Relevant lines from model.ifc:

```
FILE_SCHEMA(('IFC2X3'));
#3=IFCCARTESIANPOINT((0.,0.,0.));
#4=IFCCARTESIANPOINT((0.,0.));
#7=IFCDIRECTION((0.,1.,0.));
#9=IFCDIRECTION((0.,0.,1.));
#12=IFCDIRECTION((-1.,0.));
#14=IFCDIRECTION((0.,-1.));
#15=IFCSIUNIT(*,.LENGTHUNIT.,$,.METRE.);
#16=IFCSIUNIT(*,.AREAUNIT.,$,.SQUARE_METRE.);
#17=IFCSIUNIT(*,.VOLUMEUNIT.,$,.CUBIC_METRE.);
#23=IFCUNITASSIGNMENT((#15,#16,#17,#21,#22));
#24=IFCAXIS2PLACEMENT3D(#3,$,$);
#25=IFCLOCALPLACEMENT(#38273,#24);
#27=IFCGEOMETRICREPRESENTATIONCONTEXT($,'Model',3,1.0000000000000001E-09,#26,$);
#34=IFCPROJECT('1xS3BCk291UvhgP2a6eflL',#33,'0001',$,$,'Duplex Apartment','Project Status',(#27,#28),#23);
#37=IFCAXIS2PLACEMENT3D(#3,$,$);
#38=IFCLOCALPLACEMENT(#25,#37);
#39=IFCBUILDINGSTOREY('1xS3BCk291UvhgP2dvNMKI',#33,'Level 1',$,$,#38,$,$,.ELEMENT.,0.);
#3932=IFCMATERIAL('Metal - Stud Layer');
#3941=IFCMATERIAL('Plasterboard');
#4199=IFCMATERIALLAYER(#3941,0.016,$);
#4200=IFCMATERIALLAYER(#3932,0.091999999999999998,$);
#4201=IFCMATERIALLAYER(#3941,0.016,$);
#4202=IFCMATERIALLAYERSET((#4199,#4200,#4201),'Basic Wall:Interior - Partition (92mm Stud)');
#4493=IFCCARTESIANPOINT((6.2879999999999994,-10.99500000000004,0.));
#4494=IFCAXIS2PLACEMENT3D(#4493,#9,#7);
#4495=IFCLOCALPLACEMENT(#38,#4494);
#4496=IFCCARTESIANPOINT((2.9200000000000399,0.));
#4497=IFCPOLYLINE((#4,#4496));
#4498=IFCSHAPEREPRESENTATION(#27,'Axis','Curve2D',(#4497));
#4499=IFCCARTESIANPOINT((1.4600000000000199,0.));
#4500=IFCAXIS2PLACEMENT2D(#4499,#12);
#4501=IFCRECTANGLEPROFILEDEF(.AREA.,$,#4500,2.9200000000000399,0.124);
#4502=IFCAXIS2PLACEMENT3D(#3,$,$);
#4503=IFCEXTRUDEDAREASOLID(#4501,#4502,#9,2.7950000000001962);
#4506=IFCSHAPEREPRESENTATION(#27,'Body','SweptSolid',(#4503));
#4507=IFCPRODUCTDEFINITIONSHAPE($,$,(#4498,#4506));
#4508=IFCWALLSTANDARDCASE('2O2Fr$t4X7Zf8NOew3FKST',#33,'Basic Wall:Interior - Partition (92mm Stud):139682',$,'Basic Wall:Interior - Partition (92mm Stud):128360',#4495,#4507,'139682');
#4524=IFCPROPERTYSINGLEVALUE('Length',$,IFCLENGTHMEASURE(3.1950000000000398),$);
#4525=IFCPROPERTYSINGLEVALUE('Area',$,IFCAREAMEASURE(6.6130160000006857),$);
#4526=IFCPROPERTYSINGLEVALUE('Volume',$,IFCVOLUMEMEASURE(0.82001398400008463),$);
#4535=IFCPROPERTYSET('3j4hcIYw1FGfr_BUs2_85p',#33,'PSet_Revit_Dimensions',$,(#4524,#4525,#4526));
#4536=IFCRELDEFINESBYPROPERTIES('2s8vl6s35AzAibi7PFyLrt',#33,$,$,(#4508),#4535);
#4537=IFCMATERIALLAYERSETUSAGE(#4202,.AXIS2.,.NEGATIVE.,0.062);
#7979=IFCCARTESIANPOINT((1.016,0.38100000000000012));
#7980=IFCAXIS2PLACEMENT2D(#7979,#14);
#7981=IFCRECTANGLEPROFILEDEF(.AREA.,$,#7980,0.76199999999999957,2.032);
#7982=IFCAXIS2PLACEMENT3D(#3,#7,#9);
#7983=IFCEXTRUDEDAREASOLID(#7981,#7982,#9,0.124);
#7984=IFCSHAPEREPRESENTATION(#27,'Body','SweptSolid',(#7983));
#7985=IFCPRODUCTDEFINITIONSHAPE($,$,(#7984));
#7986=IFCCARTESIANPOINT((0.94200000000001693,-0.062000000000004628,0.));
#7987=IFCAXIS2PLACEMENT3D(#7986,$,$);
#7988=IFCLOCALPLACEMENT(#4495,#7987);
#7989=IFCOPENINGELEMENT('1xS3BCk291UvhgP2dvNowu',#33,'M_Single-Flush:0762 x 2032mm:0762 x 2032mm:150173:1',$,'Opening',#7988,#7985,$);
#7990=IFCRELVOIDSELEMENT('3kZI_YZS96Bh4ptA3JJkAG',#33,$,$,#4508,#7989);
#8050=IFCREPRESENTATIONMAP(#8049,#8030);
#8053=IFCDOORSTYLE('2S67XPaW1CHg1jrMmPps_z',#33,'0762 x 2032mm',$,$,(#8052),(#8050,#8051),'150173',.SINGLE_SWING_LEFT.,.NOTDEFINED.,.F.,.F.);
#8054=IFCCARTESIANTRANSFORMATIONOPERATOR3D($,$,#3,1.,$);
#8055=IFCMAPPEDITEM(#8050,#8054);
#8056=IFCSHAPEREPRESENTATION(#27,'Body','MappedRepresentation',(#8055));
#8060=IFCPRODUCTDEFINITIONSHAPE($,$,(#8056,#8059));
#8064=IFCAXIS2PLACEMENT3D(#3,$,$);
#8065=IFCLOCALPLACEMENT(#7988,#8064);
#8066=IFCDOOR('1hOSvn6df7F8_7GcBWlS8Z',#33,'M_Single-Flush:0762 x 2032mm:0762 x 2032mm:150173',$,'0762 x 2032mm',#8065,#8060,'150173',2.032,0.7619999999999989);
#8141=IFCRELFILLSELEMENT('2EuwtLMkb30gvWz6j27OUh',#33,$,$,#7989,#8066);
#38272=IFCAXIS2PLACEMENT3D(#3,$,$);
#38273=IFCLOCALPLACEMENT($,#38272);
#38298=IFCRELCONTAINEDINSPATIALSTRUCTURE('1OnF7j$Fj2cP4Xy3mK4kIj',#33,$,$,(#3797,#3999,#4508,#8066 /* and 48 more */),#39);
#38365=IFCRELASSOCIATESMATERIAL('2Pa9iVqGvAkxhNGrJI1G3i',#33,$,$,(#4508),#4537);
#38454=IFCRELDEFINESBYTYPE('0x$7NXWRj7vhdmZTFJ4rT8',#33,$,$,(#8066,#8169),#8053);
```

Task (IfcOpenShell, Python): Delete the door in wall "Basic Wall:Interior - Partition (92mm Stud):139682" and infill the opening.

```python
import ifcopenshell
import ifcopenshell.api.feature
import ifcopenshell.api.pset
import ifcopenshell.api.root
import ifcopenshell.geom
import ifcopenshell.util.element
import ifcopenshell.util.shape
import ifcopenshell.util.unit

model = ifcopenshell.open("model.ifc")
area_scale = ifcopenshell.util.unit.calculate_unit_scale(model, "AREAUNIT")
volume_scale = ifcopenshell.util.unit.calculate_unit_scale(model, "VOLUMEUNIT")
settings = ifcopenshell.geom.settings()


def volume(element):
    """Net volume in cubic metres, openings subtracted."""
    shape = ifcopenshell.geom.create_shape(settings, element)
    return ifcopenshell.util.shape.get_volume(shape.geometry)


door = model.by_guid("1hOSvn6df7F8_7GcBWlS8Z")
opening = door.FillsVoids[0].RelatingOpeningElement
wall = opening.VoidsElements[0].RelatingBuildingElement
before = volume(wall)

ifcopenshell.api.root.remove_product(model, product=door)
ifcopenshell.api.feature.remove_feature(model, feature=opening)

after = volume(wall)
thickness = 0.124  # wall thickness in metres

# Update the wall's stored quantities.
pset = model.by_id(ifcopenshell.util.element.get_pset(wall, "PSet_Revit_Dimensions", should_inherit=False)["id"])
ifcopenshell.api.pset.edit_pset(model, pset=pset, properties={
    "Area": model.create_entity("IfcAreaMeasure", after / thickness / area_scale),
    "Volume": model.create_entity("IfcVolumeMeasure", after / volume_scale),
})

print(f"wall volume {before:.3f} -> {after:.3f} m3")

model.write("model-out.ifc")
```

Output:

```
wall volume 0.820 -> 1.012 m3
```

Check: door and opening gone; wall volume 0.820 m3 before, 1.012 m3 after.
